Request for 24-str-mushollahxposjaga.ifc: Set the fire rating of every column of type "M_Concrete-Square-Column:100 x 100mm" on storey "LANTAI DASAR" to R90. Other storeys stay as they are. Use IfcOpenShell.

First a look at what the model holds.

```python
import ifcopenshell
import ifcopenshell.util.element

model = ifcopenshell.open("24-str-mushollahxposjaga.ifc")
print(model.schema)
storey = next(s for s in model.by_type("IfcBuildingStorey") if s.Name == "LANTAI DASAR")
columns = [e for e in ifcopenshell.util.element.get_decomposition(storey) if e.is_a("IfcColumn")]
seen = {}
for e in columns:
    element_type = ifcopenshell.util.element.get_type(e)
    key = (element_type.Name if element_type != e and element_type else None, ifcopenshell.util.element.get_pset(e, "Pset_ColumnCommon", "FireRating"))
    seen[key] = seen.get(key, 0) + 1
for (name, value), count in sorted(seen.items(), key=str):
    print(count, "x", name, "|", value)
```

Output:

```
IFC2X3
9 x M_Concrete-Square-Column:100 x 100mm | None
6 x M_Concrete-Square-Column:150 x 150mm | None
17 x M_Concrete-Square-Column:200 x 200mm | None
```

```python
import ifcopenshell
import ifcopenshell.api.pset
import ifcopenshell.util.element

model = ifcopenshell.open("24-str-mushollahxposjaga.ifc")

storey = next(s for s in model.by_type("IfcBuildingStorey") if s.Name == "LANTAI DASAR")
columns = [e for e in ifcopenshell.util.element.get_decomposition(storey) if e.is_a("IfcColumn")]

count = 0
for e in columns:
    element_type = ifcopenshell.util.element.get_type(e)
    if element_type in (None, e) or element_type.Name != "M_Concrete-Square-Column:100 x 100mm":
        continue
    # add_pset returns the element's existing set when there is one.
    pset = ifcopenshell.api.pset.add_pset(model, product=e, name="Pset_ColumnCommon")
    ifcopenshell.api.pset.edit_pset(model, pset=pset, properties={"FireRating": "R90"})
    count += 1

print(count, "columns updated")

model.write("24-str-mushollahxposjaga_v2.ifc")
```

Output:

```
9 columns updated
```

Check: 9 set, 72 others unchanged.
